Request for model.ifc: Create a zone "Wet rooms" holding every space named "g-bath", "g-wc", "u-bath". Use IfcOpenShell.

First a look at what the model holds.

```python
import ifcopenshell

model = ifcopenshell.open("model.ifc")
print(model.schema)
seen = {}
for space in model.by_type("IfcSpace"):
    seen[space.LongName] = seen.get(space.LongName, 0) + 1
for name, count in sorted(seen.items(), key=str):
    print(count, "x", name)
print("zones:", [z.Name for z in model.by_type("IfcZone")][:20])
```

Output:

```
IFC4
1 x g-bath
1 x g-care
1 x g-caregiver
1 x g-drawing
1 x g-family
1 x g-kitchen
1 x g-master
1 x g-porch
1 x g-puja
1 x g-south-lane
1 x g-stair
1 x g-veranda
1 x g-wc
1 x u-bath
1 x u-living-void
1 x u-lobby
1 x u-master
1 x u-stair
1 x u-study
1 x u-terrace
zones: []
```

```python
import ifcopenshell
import ifcopenshell.api.group
import ifcopenshell.api.root

model = ifcopenshell.open("model.ifc")

names = {"g-bath", "g-wc", "u-bath"}
spaces = [s for s in model.by_type("IfcSpace") if s.LongName in names]

zone = ifcopenshell.api.root.create_entity(model, ifc_class="IfcZone", name="Wet rooms")
ifcopenshell.api.group.assign_group(model, products=spaces, group=zone)
print(len(spaces), "spaces in", zone.Name)

model.write("model-out.ifc")
```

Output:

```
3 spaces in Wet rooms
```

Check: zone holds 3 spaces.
